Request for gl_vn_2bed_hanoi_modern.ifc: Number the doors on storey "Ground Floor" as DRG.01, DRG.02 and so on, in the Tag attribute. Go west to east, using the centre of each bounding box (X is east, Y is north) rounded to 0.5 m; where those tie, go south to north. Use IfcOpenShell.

First a look at what the model holds.

```python
import ifcopenshell
import ifcopenshell.util.element
import ifcopenshell.util.placement

model = ifcopenshell.open("gl_vn_2bed_hanoi_modern.ifc")
print(model.schema)
storey = next(s for s in model.by_type("IfcBuildingStorey") if s.Name == "Ground Floor")
doors = [e for e in ifcopenshell.util.element.get_decomposition(storey) if e.is_a("IfcDoor")]
for e in sorted(doors, key=lambda e: e.id()):
    origin = ifcopenshell.util.placement.get_local_placement(e.ObjectPlacement)[:3, 3]
    print(e.id(), e.Tag, e.Name, origin.round(2) + 0.0, sep=" | ")
```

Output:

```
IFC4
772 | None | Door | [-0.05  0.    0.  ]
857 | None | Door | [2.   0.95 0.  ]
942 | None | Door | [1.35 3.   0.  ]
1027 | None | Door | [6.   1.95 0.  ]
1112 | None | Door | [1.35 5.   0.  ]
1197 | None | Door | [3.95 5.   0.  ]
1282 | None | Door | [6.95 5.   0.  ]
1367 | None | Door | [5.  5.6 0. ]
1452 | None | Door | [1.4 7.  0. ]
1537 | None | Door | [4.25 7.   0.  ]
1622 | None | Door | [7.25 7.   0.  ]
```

```python
import ifcopenshell
import ifcopenshell.geom
import ifcopenshell.util.element
import ifcopenshell.util.shape

model = ifcopenshell.open("gl_vn_2bed_hanoi_modern.ifc")
settings = ifcopenshell.geom.settings()
settings.set("use-world-coords", True)


def centre(element):
    shape = ifcopenshell.geom.create_shape(settings, element)
    return ifcopenshell.util.shape.get_bbox_centroid(shape.geometry)


storey = next(s for s in model.by_type("IfcBuildingStorey") if s.Name == "Ground Floor")
doors = [e for e in ifcopenshell.util.element.get_decomposition(storey) if e.is_a("IfcDoor")]

# Insertion points can sit at a corner or the storey origin, so sort by the geometry (in metres).
centres = {e: centre(e) for e in doors}
doors.sort(key=lambda e: (round(centres[e][0] / 0.5), centres[e][1]))

for i, e in enumerate(doors, start=1):
    number = f"DRG.{i:02d}"
    e.Tag = number
    print(e.id(), number)

model.write("gl_vn_2bed_hanoi_modern_rev.ifc")
```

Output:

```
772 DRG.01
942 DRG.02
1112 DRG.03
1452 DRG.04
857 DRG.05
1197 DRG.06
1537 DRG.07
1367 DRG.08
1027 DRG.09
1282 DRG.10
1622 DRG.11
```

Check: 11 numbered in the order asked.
